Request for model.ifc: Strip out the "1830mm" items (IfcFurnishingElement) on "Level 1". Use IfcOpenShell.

First a look at what the model holds.

```python
import ifcopenshell
import ifcopenshell.util.element

model = ifcopenshell.open("model.ifc")
print(model.schema)
storey = next(s for s in model.by_type("IfcBuildingStorey") if s.Name == "Level 1")
furniture = [e for e in ifcopenshell.util.element.get_decomposition(storey) if e.is_a("IfcFurnishingElement")]
seen = {}
for e in furniture:
    element_type = ifcopenshell.util.element.get_type(e)
    name = element_type.Name if element_type not in (None, e) else None
    seen[name] = seen.get(name, 0) + 1
for name, count in sorted(seen.items(), key=str):
    print(count, "x", name)
```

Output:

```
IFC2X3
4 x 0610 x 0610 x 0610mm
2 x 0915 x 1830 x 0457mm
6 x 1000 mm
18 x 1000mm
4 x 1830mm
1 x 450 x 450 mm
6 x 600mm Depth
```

```python
import ifcopenshell
import ifcopenshell.api.root
import ifcopenshell.util.element

model = ifcopenshell.open("model.ifc")

storey = next(s for s in model.by_type("IfcBuildingStorey") if s.Name == "Level 1")
furniture = [e for e in ifcopenshell.util.element.get_decomposition(storey) if e.is_a("IfcFurnishingElement")]
targets = [e for e in furniture if (t := ifcopenshell.util.element.get_type(e)) not in (None, e) and t.Name == "1830mm"]

for e in targets:
    ifcopenshell.api.root.remove_product(model, product=e)
print(len(targets), "removed")

model.write("model_updated.ifc")
```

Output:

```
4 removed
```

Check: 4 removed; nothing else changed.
